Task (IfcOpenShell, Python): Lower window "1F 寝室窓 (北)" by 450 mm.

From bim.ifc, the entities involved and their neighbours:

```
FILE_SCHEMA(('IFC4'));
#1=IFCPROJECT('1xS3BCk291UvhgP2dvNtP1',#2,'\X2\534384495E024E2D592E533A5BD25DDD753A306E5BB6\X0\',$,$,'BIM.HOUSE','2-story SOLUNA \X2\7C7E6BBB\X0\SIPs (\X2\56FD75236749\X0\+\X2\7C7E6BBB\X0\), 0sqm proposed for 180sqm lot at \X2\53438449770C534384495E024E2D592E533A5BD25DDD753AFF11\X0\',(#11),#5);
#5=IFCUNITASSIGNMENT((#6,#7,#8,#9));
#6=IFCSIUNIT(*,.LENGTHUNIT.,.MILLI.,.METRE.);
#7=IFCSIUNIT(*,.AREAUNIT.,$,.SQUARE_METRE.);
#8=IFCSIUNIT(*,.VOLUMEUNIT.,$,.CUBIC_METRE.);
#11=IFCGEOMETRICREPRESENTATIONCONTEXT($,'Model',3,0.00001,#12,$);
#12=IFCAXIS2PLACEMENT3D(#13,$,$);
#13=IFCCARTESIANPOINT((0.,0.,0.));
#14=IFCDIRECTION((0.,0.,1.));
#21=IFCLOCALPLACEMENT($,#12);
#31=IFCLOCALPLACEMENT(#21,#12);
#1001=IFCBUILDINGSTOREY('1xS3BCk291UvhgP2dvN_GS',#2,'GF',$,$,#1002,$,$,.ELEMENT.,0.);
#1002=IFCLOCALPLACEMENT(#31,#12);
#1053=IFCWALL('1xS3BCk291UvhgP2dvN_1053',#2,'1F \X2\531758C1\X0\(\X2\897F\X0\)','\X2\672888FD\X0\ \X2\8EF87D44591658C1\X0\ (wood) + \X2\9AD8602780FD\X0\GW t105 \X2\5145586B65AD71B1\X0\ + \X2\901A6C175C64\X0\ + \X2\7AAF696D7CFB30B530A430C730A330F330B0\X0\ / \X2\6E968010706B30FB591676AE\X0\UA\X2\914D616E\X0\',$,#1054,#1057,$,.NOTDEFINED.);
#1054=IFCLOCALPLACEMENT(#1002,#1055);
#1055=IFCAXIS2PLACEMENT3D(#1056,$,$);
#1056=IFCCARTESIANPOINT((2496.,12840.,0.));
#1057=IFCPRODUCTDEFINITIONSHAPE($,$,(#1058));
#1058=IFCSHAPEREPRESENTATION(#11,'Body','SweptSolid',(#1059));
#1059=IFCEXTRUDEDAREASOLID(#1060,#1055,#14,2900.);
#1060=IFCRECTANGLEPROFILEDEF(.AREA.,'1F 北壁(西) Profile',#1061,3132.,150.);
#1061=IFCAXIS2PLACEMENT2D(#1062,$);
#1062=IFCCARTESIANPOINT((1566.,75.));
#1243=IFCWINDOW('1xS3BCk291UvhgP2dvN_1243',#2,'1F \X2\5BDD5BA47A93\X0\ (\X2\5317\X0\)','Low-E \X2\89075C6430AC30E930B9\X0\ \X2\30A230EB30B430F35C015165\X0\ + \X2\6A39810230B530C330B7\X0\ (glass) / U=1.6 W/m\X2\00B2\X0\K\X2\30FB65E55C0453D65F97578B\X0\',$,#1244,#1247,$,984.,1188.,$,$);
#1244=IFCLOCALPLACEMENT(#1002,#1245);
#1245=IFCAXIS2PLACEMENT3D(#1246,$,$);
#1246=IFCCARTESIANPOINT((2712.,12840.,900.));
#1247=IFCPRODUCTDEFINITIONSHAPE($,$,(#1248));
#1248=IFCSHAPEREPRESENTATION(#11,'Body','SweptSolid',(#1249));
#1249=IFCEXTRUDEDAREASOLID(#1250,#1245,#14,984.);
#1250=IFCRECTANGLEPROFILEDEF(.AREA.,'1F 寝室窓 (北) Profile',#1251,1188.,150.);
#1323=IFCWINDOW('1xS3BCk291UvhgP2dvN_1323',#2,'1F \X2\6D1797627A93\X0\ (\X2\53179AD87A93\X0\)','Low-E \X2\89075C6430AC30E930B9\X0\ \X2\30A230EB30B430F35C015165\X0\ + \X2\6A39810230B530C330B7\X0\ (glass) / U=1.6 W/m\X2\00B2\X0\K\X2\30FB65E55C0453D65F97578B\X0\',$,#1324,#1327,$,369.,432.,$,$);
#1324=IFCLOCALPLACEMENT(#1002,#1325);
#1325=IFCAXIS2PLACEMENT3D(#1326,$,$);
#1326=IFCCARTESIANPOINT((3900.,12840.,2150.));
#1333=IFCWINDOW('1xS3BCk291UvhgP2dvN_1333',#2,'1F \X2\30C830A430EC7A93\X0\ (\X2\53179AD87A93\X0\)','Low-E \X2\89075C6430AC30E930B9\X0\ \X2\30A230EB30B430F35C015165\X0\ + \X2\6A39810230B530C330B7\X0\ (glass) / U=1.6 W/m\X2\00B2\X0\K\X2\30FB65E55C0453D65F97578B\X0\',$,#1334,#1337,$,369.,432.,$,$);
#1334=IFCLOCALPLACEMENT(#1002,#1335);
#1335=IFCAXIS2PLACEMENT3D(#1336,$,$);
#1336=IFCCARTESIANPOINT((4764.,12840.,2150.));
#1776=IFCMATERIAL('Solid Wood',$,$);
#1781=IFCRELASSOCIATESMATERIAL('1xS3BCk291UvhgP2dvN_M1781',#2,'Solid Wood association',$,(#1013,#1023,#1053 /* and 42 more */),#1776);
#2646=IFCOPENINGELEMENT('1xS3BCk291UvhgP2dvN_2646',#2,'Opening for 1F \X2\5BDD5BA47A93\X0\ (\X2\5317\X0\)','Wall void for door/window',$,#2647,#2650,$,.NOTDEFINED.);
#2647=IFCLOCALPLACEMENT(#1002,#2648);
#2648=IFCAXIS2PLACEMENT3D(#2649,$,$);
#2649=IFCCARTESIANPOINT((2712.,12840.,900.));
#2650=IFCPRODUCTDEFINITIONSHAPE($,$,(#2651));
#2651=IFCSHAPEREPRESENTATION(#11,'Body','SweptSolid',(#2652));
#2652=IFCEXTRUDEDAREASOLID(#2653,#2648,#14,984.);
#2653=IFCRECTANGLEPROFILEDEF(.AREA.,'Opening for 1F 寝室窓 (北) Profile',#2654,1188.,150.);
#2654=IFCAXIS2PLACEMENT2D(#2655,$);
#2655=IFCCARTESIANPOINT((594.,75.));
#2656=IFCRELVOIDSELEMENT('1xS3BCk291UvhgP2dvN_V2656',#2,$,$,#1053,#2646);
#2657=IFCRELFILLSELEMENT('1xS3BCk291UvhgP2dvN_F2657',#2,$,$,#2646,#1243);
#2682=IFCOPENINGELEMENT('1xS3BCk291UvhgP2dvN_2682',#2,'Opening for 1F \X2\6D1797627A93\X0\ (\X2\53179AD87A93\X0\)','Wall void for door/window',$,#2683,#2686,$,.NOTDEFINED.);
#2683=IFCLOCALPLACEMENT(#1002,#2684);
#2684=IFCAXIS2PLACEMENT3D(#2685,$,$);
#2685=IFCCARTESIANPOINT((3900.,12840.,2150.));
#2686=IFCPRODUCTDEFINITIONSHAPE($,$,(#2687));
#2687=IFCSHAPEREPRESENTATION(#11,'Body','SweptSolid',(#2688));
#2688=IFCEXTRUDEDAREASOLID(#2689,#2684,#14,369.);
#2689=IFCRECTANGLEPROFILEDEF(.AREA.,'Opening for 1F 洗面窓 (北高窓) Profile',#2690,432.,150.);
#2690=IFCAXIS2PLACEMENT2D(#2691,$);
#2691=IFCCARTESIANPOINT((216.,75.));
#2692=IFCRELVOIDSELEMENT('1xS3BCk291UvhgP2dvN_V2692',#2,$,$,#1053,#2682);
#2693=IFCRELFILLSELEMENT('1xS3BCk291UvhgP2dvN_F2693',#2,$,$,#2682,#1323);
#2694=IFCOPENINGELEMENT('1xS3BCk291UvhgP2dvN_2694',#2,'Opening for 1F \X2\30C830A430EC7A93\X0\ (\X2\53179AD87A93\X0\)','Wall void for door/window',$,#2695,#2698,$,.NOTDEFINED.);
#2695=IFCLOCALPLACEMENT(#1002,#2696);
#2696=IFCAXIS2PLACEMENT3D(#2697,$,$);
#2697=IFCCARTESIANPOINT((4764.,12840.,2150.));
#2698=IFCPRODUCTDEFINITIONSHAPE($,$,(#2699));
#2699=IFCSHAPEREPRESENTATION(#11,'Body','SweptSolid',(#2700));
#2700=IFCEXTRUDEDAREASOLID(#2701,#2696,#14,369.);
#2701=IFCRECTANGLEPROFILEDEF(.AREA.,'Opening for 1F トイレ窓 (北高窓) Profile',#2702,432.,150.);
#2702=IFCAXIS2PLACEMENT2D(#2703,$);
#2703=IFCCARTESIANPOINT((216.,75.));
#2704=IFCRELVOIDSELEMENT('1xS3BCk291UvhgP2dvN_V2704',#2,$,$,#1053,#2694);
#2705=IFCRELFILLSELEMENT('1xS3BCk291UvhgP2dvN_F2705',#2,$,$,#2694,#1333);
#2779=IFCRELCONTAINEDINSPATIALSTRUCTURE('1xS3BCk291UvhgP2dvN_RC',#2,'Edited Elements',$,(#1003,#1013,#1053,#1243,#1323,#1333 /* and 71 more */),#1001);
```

```python
import numpy as np
import ifcopenshell
import ifcopenshell.api.geometry
import ifcopenshell.util.placement
import ifcopenshell.util.unit

model = ifcopenshell.open("bim.ifc")
unit_scale = ifcopenshell.util.unit.calculate_unit_scale(model)

window = model.by_id(1243)
opening = window.FillsVoids[0].RelatingOpeningElement
dz = -450.0

shift = np.array([0.0, 0.0, dz])
# The window is not placed relative to its opening, so move both.
for product in (opening, window):
    matrix = ifcopenshell.util.placement.get_local_placement(product.ObjectPlacement)
    matrix[:3, 3] += shift
    ifcopenshell.api.geometry.edit_object_placement(model, product=product, matrix=matrix, is_si=False)

print(f"moved by {dz * unit_scale:+.3f} m")

model.write("bim_edited.ifc")
```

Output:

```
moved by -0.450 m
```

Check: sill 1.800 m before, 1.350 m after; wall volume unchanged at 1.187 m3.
